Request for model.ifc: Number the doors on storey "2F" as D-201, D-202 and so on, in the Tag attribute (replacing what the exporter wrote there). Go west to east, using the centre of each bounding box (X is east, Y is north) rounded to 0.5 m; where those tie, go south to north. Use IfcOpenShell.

First a look at what the model holds.

```python
import ifcopenshell
import ifcopenshell.util.element
import ifcopenshell.util.placement

model = ifcopenshell.open("model.ifc")
print(model.schema)
storey = next(s for s in model.by_type("IfcBuildingStorey") if s.Name == "2F")
doors = [e for e in ifcopenshell.util.element.get_decomposition(storey) if e.is_a("IfcDoor")]
for e in sorted(doors, key=lambda e: e.id()):
    origin = ifcopenshell.util.placement.get_local_placement(e.ObjectPlacement)[:3, 3]
    print(e.id(), e.Tag, e.Name, origin.round(2) + 0.0, sep=" | ")
```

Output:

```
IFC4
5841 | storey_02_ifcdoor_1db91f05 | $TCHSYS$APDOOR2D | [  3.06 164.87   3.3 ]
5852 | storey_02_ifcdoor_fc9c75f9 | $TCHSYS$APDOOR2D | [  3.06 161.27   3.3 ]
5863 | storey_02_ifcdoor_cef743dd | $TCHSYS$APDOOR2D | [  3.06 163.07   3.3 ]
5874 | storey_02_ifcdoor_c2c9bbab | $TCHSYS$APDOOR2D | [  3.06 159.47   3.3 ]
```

```python
import ifcopenshell
import ifcopenshell.geom
import ifcopenshell.util.element
import ifcopenshell.util.shape

model = ifcopenshell.open("model.ifc")
settings = ifcopenshell.geom.settings()
settings.set("use-world-coords", True)


def centre(element):
    shape = ifcopenshell.geom.create_shape(settings, element)
    return ifcopenshell.util.shape.get_bbox_centroid(shape.geometry)


storey = next(s for s in model.by_type("IfcBuildingStorey") if s.Name == "2F")
doors = [e for e in ifcopenshell.util.element.get_decomposition(storey) if e.is_a("IfcDoor")]

# Insertion points can sit at a corner or the storey origin, so sort by the geometry (in metres).
centres = {e: centre(e) for e in doors}
doors.sort(key=lambda e: (round(centres[e][0] / 0.5), centres[e][1]))

for i, e in enumerate(doors, start=1):
    number = f"D-2{i:02d}"
    e.Tag = number
    print(e.id(), number)

model.write("model_rev.ifc")
```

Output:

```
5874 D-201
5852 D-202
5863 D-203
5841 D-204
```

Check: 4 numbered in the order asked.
